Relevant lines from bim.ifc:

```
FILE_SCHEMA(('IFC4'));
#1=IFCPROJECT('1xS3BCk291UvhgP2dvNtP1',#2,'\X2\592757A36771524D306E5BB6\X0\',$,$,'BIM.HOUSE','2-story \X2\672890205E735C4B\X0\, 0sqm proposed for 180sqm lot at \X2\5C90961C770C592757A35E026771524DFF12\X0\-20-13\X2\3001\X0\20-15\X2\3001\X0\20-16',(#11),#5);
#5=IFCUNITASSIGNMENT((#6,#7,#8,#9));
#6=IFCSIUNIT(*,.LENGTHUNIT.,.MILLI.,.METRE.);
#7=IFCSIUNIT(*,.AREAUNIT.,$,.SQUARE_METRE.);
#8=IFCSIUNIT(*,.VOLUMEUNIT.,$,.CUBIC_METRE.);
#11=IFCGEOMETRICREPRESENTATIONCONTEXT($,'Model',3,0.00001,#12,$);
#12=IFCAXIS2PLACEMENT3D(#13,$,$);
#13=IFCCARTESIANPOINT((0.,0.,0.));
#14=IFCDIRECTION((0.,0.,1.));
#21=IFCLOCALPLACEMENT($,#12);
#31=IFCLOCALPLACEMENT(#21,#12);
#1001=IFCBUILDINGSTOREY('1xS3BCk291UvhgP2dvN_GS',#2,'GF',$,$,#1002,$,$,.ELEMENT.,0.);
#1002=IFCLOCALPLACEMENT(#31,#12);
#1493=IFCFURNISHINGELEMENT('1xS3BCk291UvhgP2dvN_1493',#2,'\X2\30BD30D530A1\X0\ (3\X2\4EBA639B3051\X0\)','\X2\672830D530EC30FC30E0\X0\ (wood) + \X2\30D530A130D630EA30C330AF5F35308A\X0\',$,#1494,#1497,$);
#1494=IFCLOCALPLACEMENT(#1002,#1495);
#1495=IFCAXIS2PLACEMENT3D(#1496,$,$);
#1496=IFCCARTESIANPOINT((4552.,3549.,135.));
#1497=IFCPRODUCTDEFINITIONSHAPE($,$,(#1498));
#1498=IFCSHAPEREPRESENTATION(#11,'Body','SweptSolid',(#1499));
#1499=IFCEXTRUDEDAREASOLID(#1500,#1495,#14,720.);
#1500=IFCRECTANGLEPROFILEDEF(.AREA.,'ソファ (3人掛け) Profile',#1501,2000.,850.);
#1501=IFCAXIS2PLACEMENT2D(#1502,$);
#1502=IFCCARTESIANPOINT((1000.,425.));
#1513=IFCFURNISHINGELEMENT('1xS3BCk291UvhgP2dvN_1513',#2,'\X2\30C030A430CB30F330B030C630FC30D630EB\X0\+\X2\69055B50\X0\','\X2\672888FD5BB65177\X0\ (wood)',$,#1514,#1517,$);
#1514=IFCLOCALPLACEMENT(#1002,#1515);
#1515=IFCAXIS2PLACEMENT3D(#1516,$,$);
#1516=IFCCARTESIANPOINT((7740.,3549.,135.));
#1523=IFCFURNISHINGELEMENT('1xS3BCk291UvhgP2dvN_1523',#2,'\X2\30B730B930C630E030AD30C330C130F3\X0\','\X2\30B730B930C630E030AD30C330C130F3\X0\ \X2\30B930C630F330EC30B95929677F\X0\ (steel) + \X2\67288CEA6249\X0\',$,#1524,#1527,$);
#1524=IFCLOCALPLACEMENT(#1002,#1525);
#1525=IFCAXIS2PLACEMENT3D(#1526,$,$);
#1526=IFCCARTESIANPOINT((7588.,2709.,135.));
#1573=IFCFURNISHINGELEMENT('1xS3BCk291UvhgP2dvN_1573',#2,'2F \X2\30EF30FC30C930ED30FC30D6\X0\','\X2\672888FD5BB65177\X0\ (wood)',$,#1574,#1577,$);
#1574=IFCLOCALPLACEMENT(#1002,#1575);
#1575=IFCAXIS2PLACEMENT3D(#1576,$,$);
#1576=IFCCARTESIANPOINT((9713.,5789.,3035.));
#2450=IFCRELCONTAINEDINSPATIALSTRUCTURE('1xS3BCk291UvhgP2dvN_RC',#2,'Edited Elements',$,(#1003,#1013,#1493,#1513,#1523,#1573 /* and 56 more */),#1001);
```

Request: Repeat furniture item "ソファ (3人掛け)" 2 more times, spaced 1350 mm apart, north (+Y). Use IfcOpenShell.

```python
import numpy as np
import ifcopenshell
import ifcopenshell.api.geometry
import ifcopenshell.api.root
import ifcopenshell.util.element
import ifcopenshell.util.placement
import ifcopenshell.util.unit

model = ifcopenshell.open("bim.ifc")
unit_scale = ifcopenshell.util.unit.calculate_unit_scale(model)


def reuse_history(source, copy):
    """copy_class also copies each property set's owner history, people and application; keep the originals."""
    for rel in copy.IsDefinedBy:
        if rel.is_a("IfcRelDefinesByProperties") and (history := rel.RelatingPropertyDefinition.OwnerHistory):
            rel.RelatingPropertyDefinition.OwnerHistory = source.OwnerHistory
            ifcopenshell.util.element.remove_deep2(model, history)


source = model.by_guid("1xS3BCk291UvhgP2dvN_1493")
base = ifcopenshell.util.placement.get_local_placement(source.ObjectPlacement)
step = np.array([0.0, 1.0, 0.0]) * 1.35 / unit_scale

for i in range(1, 3):
    copy = ifcopenshell.api.root.copy_class(model, product=source)
    copy.Representation = ifcopenshell.util.element.copy_deep(
        model, source.Representation, exclude=["IfcGeometricRepresentationContext", "IfcRepresentationMap"]
    )
    reuse_history(source, copy)
    matrix = base.copy()
    matrix[:3, 3] += i * step
    print("added at", matrix[:3, 3].round(3) + 0.0)
    ifcopenshell.api.geometry.edit_object_placement(model, product=copy, matrix=matrix, is_si=False)

model.write("bim_rev.ifc")
```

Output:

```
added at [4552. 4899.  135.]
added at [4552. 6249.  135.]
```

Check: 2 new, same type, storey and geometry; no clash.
